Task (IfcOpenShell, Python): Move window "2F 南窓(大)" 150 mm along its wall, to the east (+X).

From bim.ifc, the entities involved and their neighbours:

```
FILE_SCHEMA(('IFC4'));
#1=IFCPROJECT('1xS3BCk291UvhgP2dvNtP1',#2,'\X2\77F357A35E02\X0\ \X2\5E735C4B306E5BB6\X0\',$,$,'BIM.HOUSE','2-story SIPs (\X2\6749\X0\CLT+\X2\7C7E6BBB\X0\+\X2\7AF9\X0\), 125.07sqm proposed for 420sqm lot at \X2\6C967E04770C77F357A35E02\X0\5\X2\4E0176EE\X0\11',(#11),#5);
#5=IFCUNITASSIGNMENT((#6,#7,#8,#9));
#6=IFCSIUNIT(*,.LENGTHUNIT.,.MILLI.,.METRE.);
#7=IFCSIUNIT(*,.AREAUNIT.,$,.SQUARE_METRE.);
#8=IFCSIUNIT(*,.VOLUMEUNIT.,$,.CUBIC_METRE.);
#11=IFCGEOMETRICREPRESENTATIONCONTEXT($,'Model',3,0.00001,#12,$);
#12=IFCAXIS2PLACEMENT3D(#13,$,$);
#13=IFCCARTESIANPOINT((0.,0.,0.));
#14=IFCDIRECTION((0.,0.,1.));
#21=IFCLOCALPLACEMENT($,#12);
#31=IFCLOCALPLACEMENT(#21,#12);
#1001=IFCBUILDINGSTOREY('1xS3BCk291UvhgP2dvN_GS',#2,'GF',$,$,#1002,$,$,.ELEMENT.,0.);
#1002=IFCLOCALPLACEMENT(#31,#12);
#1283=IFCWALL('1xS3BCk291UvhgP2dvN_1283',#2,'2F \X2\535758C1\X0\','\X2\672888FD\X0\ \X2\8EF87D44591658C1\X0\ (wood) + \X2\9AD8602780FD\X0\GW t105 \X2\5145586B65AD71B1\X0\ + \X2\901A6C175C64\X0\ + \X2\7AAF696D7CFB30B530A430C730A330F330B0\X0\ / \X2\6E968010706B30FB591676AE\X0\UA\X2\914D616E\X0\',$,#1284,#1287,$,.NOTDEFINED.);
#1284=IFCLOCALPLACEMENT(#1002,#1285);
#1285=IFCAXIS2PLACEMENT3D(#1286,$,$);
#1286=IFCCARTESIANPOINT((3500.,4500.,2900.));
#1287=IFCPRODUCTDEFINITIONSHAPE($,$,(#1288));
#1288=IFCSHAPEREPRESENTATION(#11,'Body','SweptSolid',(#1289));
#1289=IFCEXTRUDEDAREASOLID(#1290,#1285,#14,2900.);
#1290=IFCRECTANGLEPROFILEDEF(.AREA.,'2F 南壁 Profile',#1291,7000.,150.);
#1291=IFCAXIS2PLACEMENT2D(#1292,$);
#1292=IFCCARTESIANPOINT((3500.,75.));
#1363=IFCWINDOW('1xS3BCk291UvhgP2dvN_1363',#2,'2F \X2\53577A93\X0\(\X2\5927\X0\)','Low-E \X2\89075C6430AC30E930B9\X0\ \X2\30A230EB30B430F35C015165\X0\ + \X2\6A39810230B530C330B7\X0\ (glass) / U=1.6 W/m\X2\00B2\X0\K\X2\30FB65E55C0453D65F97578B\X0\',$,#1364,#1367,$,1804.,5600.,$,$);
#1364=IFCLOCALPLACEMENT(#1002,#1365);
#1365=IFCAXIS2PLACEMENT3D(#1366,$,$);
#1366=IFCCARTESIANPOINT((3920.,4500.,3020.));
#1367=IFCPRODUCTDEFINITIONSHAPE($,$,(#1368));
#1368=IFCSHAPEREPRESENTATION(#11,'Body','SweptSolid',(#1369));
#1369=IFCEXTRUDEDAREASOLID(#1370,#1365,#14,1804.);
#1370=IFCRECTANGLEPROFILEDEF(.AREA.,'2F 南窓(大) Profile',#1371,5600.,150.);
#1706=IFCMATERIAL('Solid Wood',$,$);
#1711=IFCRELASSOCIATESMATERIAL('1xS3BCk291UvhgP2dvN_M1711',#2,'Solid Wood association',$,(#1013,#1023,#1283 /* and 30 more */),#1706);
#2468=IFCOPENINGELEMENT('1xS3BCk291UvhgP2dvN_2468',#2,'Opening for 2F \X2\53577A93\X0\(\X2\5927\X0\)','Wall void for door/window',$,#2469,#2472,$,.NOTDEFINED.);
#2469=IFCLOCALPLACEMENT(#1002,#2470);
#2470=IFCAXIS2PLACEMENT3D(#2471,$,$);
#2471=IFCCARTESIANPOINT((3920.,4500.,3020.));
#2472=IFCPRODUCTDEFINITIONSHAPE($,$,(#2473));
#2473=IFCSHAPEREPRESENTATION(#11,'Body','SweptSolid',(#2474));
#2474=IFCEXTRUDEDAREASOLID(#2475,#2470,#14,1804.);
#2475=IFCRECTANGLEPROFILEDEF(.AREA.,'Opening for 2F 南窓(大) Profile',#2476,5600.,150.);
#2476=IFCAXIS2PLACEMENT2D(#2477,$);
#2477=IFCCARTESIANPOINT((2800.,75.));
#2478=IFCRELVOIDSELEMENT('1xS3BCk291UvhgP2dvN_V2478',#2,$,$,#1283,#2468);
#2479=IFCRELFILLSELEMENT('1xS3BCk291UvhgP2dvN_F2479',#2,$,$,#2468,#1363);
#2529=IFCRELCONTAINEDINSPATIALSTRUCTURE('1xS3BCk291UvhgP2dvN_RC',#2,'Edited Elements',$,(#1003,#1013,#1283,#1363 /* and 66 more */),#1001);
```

```python
import ifcopenshell
import ifcopenshell.api.geometry
import ifcopenshell.util.placement
import ifcopenshell.util.unit

model = ifcopenshell.open("bim.ifc")
unit_scale = ifcopenshell.util.unit.calculate_unit_scale(model)

window = model.by_guid("1xS3BCk291UvhgP2dvN_1363")
opening = window.FillsVoids[0].RelatingOpeningElement
wall = opening.VoidsElements[0].RelatingBuildingElement

wall_matrix = ifcopenshell.util.placement.get_local_placement(wall.ObjectPlacement)
shift = wall_matrix[:3, 0] * 0.15 / unit_scale
before = ifcopenshell.util.placement.get_local_placement(window.ObjectPlacement)[:3, 3].copy()

# The window is not placed relative to its opening, so move both.
for product in (opening, window):
    matrix = ifcopenshell.util.placement.get_local_placement(product.ObjectPlacement)
    matrix[:3, 3] += shift
    ifcopenshell.api.geometry.edit_object_placement(model, product=product, matrix=matrix, is_si=False)

after = ifcopenshell.util.placement.get_local_placement(window.ObjectPlacement)[:3, 3]
print("window moved by", (after - before).round(3) + 0.0)

model.write("bim_updated.ifc")
```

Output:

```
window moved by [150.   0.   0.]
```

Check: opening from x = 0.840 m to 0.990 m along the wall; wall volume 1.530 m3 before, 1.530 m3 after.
